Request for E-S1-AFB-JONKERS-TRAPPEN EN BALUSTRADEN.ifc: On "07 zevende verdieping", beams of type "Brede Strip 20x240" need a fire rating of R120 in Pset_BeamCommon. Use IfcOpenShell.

First a look at what the model holds.

```python
import ifcopenshell
import ifcopenshell.util.element

model = ifcopenshell.open("E-S1-AFB-JONKERS-TRAPPEN EN BALUSTRADEN.ifc")
print(model.schema)
storey = next(s for s in model.by_type("IfcBuildingStorey") if s.Name == "07 zevende verdieping")
beams = [e for e in ifcopenshell.util.element.get_decomposition(storey) if e.is_a("IfcBeam")]
seen = {}
for e in beams:
    element_type = ifcopenshell.util.element.get_type(e)
    key = (element_type.Name if element_type != e and element_type else None, ifcopenshell.util.element.get_pset(e, "Pset_BeamCommon", "FireRating"))
    seen[key] = seen.get(key, 0) + 1
for (name, value), count in sorted(seen.items(), key=str):
    print(count, "x", name, "|", value)
```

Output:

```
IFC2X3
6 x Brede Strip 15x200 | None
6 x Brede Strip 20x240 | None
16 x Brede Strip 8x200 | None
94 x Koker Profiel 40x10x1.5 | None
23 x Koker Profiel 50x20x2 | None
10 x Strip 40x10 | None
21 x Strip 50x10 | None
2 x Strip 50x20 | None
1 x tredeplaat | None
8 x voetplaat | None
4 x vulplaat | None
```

```python
import ifcopenshell
import ifcopenshell.api.pset
import ifcopenshell.util.element

model = ifcopenshell.open("E-S1-AFB-JONKERS-TRAPPEN EN BALUSTRADEN.ifc")

storey = next(s for s in model.by_type("IfcBuildingStorey") if s.Name == "07 zevende verdieping")
beams = [e for e in ifcopenshell.util.element.get_decomposition(storey) if e.is_a("IfcBeam")]

count = 0
for e in beams:
    element_type = ifcopenshell.util.element.get_type(e)
    if element_type in (None, e) or element_type.Name != "Brede Strip 20x240":
        continue
    # add_pset returns the element's existing set when there is one.
    pset = ifcopenshell.api.pset.add_pset(model, product=e, name="Pset_BeamCommon")
    ifcopenshell.api.pset.edit_pset(model, pset=pset, properties={"FireRating": "R120"})
    count += 1

print(count, "beams updated")

model.write("E-S1-AFB-JONKERS-TRAPPEN EN BALUSTRADEN_rev.ifc")
```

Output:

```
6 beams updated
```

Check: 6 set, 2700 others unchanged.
